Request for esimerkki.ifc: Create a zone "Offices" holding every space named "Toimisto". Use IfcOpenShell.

First a look at what the model holds.

```python
import ifcopenshell

model = ifcopenshell.open("esimerkki.ifc")
print(model.schema)
seen = {}
for space in model.by_type("IfcSpace"):
    seen[space.LongName] = seen.get(space.LongName, 0) + 1
for name, count in sorted(seen.items(), key=str):
    print(count, "x", name)
print("zones:", [z.Name for z in model.by_type("IfcZone")][:20])
```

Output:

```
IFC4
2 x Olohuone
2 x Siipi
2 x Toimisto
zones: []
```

```python
import ifcopenshell
import ifcopenshell.api.group
import ifcopenshell.api.root

model = ifcopenshell.open("esimerkki.ifc")

names = {"Toimisto"}
spaces = [s for s in model.by_type("IfcSpace") if s.LongName in names]

zone = ifcopenshell.api.root.create_entity(model, ifc_class="IfcZone", name="Offices")
ifcopenshell.api.group.assign_group(model, products=spaces, group=zone)
print(len(spaces), "spaces in", zone.Name)

model.write("esimerkki_v2.ifc")
```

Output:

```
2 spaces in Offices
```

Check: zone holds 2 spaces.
